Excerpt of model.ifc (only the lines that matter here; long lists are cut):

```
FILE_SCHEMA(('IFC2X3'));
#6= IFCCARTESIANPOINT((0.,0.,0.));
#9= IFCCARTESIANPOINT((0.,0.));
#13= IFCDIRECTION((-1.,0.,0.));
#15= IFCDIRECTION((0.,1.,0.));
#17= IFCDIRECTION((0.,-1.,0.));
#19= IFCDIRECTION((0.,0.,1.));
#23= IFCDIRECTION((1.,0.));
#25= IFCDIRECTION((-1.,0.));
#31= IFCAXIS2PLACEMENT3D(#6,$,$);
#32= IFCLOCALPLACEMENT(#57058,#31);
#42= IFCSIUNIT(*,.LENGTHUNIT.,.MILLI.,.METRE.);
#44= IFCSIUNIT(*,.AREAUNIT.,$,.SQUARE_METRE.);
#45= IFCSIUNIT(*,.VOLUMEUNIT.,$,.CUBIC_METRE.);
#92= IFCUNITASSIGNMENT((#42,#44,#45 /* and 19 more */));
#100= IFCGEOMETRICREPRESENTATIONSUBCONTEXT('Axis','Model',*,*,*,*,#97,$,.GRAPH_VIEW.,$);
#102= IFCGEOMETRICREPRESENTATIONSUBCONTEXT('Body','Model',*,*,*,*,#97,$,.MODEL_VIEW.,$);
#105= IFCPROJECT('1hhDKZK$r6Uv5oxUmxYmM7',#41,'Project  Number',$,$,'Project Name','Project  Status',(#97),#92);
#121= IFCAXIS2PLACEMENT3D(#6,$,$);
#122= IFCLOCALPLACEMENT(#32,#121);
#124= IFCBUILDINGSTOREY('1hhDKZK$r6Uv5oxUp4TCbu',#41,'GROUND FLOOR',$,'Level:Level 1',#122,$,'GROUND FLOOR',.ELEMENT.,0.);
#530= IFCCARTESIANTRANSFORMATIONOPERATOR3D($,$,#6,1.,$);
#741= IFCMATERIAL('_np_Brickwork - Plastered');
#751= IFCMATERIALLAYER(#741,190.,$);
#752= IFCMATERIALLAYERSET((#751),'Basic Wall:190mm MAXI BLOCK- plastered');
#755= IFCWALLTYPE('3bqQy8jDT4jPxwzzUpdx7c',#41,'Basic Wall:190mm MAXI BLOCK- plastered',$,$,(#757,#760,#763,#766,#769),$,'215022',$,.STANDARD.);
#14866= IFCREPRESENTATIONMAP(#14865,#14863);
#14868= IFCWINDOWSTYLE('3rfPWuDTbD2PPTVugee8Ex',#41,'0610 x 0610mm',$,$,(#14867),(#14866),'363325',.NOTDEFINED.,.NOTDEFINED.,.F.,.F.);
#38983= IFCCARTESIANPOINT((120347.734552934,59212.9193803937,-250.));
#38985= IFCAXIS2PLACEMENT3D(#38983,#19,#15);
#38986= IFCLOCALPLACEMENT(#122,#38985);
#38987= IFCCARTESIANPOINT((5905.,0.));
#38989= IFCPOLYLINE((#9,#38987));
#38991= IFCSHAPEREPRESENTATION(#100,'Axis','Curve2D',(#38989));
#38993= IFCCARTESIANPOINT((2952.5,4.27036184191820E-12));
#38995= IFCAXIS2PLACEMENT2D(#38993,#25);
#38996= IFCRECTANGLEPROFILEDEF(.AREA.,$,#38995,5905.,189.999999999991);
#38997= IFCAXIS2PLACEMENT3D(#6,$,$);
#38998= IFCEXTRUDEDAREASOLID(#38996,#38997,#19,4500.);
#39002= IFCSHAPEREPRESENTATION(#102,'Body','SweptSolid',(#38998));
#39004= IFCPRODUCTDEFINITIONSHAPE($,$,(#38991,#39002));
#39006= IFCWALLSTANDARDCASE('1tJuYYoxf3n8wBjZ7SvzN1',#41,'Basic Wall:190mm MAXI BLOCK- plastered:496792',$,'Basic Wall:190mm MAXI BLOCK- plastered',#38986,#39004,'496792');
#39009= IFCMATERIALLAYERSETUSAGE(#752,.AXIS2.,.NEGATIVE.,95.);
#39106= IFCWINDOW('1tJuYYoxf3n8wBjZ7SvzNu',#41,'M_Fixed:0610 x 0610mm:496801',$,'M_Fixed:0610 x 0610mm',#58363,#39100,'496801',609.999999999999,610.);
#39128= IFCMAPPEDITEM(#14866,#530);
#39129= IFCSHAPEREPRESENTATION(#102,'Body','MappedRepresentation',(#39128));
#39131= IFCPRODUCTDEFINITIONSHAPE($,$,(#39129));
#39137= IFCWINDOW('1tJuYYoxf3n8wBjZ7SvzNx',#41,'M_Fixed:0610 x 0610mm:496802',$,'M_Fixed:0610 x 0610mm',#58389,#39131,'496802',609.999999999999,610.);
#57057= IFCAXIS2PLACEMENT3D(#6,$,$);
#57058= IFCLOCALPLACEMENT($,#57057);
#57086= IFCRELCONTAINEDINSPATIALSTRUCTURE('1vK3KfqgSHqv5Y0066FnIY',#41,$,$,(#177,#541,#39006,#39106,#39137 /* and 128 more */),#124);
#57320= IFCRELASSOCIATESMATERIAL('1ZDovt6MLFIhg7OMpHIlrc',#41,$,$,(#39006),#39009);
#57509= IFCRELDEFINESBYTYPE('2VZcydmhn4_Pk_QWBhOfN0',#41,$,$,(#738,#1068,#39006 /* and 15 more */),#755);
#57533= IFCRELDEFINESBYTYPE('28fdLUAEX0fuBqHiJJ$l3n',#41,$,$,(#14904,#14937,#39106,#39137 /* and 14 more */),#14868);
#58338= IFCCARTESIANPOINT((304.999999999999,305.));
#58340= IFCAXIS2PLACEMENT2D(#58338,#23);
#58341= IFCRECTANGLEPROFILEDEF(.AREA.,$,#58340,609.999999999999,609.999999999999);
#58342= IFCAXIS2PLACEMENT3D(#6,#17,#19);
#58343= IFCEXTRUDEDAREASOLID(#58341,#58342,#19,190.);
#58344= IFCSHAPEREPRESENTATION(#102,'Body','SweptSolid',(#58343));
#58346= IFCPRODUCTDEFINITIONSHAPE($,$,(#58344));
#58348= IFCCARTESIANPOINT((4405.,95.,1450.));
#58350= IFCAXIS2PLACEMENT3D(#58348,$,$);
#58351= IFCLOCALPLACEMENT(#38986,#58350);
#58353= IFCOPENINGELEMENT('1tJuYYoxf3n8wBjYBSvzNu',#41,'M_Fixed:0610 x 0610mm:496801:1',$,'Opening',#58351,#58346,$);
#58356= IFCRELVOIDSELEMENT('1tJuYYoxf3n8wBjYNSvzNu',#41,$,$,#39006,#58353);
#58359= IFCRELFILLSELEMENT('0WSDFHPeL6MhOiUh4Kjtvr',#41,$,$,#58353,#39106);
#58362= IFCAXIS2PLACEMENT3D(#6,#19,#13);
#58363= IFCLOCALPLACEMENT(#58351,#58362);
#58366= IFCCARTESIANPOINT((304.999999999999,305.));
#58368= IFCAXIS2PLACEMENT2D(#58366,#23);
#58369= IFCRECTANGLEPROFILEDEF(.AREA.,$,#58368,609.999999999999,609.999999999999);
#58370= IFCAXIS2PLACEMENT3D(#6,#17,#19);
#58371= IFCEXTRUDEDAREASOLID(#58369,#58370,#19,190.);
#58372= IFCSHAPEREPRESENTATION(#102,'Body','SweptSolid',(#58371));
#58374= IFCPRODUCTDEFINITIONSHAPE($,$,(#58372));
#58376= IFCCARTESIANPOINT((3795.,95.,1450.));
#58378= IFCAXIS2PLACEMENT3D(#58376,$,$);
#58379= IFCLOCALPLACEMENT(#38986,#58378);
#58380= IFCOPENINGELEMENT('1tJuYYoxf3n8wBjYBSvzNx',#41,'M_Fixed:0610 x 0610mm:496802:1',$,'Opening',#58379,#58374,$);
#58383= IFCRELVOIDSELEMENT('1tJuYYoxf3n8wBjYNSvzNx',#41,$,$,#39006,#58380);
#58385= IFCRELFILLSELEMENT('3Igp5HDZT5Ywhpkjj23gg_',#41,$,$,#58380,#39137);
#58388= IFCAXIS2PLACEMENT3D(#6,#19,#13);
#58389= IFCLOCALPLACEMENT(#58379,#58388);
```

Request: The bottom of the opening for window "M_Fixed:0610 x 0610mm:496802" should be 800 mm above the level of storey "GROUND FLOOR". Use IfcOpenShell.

```python
import numpy as np
import ifcopenshell
import ifcopenshell.api.geometry
import ifcopenshell.geom
import ifcopenshell.util.element
import ifcopenshell.util.placement
import ifcopenshell.util.shape
import ifcopenshell.util.unit

model = ifcopenshell.open("model.ifc")
unit_scale = ifcopenshell.util.unit.calculate_unit_scale(model)

window = model.by_guid("1tJuYYoxf3n8wBjZ7SvzNx")
opening = window.FillsVoids[0].RelatingOpeningElement
storey = ifcopenshell.util.element.get_container(window, ifc_class="IfcBuildingStorey")
level = ifcopenshell.util.placement.get_local_placement(storey.ObjectPlacement)[2, 3]

# The opening's origin need not be at the sill, so measure its lowest point.
shape = ifcopenshell.geom.create_shape(ifcopenshell.geom.settings(), opening)
bottom = ifcopenshell.util.shape.get_shape_bottom_elevation(shape, shape.geometry) / unit_scale
dz = level + 0.8 / unit_scale - bottom

shift = np.array([0.0, 0.0, dz])
# The window is placed relative to its opening, so it follows when the opening moves.
matrix = ifcopenshell.util.placement.get_local_placement(opening.ObjectPlacement)
matrix[:3, 3] += shift
ifcopenshell.api.geometry.edit_object_placement(
    model, product=opening, matrix=matrix, is_si=False, should_transform_children=True
)

print(f"moved by {dz * unit_scale:+.3f} m")

model.write("model_v2.ifc")
```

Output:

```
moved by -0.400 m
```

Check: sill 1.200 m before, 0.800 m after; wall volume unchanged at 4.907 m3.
